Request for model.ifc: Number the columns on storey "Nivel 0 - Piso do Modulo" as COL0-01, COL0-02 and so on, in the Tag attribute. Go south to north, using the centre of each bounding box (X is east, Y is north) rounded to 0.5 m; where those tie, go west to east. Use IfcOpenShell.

First a look at what the model holds.

```python
import ifcopenshell
import ifcopenshell.util.element
import ifcopenshell.util.placement

model = ifcopenshell.open("model.ifc")
print(model.schema)
storey = next(s for s in model.by_type("IfcBuildingStorey") if s.Name == "Nivel 0 - Piso do Modulo")
columns = [e for e in ifcopenshell.util.element.get_decomposition(storey) if e.is_a("IfcColumn")]
for e in sorted(columns, key=lambda e: e.id()):
    origin = ifcopenshell.util.placement.get_local_placement(e.ObjectPlacement)[:3, 3]
    print(e.id(), e.Tag, e.Name, origin.round(2) + 0.0, sep=" | ")
```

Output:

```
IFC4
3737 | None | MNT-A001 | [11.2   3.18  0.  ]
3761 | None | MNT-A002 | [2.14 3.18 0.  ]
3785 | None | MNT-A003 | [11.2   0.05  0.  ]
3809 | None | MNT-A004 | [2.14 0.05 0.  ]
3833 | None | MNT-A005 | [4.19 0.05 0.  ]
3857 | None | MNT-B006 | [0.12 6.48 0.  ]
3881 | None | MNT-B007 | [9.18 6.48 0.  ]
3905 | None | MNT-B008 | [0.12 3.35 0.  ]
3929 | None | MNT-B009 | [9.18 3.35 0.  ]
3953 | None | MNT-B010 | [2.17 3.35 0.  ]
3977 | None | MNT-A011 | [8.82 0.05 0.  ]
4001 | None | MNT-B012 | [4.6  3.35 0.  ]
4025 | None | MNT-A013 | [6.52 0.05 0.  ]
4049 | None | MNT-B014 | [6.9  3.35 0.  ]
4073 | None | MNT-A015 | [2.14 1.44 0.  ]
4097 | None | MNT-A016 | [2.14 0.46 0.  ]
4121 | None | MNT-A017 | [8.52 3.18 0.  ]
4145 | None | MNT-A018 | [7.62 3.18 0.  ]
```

```python
import ifcopenshell
import ifcopenshell.geom
import ifcopenshell.util.element
import ifcopenshell.util.shape

model = ifcopenshell.open("model.ifc")
settings = ifcopenshell.geom.settings()
settings.set("use-world-coords", True)


def centre(element):
    shape = ifcopenshell.geom.create_shape(settings, element)
    return ifcopenshell.util.shape.get_bbox_centroid(shape.geometry)


storey = next(s for s in model.by_type("IfcBuildingStorey") if s.Name == "Nivel 0 - Piso do Modulo")
columns = [e for e in ifcopenshell.util.element.get_decomposition(storey) if e.is_a("IfcColumn")]

# Insertion points can sit at a corner or the storey origin, so sort by the geometry (in metres).
centres = {e: centre(e) for e in columns}
columns.sort(key=lambda e: (round(centres[e][1] / 0.5), centres[e][0]))

for i, e in enumerate(columns, start=1):
    number = f"COL0-{i:02d}"
    e.Tag = number
    print(e.id(), number)

model.write("model_updated.ifc")
```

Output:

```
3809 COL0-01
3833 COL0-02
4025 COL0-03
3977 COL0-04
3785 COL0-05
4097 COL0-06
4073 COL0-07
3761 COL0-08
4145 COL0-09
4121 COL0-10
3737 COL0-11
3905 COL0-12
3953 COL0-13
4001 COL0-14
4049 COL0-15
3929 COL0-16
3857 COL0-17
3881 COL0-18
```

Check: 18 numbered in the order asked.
